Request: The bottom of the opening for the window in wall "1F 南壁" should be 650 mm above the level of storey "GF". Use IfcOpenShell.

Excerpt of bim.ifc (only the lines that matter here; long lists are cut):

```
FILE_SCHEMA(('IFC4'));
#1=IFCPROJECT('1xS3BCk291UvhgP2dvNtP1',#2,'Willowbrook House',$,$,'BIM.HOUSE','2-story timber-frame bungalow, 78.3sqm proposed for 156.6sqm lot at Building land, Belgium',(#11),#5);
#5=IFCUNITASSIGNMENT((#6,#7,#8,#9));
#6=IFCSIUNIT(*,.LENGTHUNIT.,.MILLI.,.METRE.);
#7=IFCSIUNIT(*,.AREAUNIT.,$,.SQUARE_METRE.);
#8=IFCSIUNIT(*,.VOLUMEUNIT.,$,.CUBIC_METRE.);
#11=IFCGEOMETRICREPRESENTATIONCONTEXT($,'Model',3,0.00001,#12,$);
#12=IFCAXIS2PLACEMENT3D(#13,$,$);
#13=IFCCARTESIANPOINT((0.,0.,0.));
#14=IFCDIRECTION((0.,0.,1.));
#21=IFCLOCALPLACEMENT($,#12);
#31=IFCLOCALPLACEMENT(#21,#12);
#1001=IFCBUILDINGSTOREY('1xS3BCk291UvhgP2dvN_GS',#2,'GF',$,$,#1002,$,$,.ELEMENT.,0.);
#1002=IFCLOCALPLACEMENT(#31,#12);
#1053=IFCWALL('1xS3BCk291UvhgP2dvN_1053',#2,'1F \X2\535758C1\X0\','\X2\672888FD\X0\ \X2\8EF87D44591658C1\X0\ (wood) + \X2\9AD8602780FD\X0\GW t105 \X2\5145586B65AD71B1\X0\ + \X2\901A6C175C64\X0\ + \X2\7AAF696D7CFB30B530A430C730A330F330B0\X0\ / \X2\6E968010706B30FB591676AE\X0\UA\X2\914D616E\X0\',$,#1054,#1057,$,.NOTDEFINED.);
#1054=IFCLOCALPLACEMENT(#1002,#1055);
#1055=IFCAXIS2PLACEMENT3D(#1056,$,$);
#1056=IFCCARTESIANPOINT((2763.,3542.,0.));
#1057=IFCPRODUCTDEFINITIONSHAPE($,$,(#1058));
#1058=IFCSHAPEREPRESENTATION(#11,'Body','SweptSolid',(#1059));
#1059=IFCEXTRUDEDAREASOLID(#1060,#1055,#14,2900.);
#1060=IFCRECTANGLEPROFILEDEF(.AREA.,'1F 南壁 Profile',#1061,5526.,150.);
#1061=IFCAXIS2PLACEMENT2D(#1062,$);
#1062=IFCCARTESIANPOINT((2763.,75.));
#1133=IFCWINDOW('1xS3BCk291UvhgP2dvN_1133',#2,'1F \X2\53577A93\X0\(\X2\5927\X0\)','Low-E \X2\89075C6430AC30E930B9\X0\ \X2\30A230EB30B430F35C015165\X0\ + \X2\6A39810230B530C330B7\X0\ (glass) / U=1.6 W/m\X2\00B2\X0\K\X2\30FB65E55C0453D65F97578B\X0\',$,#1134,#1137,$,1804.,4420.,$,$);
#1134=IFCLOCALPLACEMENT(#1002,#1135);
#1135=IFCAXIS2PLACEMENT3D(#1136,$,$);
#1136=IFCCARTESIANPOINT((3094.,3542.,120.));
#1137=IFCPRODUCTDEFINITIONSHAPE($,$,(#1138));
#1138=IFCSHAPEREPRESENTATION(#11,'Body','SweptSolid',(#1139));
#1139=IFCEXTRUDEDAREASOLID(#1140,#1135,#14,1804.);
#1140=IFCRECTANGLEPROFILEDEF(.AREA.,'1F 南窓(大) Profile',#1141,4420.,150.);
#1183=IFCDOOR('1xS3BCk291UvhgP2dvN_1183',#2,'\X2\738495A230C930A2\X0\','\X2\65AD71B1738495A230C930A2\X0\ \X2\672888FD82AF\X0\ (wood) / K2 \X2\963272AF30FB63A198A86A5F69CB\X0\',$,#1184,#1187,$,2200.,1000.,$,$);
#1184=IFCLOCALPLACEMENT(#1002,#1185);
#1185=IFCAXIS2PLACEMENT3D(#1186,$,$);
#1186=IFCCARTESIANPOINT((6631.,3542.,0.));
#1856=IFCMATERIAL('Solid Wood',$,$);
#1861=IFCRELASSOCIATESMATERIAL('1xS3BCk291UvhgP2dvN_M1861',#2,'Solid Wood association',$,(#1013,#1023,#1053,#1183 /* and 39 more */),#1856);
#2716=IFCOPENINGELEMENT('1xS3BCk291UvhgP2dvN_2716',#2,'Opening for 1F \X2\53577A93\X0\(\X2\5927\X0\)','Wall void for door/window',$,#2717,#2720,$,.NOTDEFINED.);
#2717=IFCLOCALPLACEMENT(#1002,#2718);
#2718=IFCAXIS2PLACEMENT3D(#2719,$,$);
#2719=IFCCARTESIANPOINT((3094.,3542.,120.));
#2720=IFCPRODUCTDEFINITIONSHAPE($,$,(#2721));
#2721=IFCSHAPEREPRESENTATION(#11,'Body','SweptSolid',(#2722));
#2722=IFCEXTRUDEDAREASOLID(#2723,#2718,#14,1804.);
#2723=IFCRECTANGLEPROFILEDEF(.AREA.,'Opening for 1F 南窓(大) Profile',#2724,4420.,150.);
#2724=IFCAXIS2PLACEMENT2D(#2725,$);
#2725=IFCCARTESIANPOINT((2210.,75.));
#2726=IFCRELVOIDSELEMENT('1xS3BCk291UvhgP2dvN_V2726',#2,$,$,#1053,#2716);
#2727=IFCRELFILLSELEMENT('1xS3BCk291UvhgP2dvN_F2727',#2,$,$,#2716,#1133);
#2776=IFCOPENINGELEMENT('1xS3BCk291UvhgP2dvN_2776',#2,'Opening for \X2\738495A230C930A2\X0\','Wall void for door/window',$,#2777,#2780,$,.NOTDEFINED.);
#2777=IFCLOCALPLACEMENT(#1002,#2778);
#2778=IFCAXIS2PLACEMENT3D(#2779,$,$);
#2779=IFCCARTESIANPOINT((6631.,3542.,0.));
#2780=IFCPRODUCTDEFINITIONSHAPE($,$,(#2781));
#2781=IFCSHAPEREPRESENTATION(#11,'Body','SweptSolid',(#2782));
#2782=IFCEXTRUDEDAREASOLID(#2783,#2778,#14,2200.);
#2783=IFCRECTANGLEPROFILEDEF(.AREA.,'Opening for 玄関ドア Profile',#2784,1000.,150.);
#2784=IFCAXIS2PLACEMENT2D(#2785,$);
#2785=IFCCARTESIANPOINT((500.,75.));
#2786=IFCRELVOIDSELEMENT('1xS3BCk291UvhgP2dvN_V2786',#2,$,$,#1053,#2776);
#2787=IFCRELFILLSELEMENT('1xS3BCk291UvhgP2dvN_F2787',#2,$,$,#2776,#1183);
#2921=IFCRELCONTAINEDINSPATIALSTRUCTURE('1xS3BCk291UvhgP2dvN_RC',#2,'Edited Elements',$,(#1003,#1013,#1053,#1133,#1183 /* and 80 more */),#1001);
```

```python
import numpy as np
import ifcopenshell
import ifcopenshell.api.geometry
import ifcopenshell.geom
import ifcopenshell.util.element
import ifcopenshell.util.placement
import ifcopenshell.util.shape
import ifcopenshell.util.unit

model = ifcopenshell.open("bim.ifc")
unit_scale = ifcopenshell.util.unit.calculate_unit_scale(model)

window = model.by_guid("1xS3BCk291UvhgP2dvN_1133")
opening = window.FillsVoids[0].RelatingOpeningElement
storey = ifcopenshell.util.element.get_container(window, ifc_class="IfcBuildingStorey")
level = ifcopenshell.util.placement.get_local_placement(storey.ObjectPlacement)[2, 3]

# The opening's origin need not be at the sill, so measure its lowest point.
shape = ifcopenshell.geom.create_shape(ifcopenshell.geom.settings(), opening)
bottom = ifcopenshell.util.shape.get_shape_bottom_elevation(shape, shape.geometry) / unit_scale
dz = level + 0.65 / unit_scale - bottom

shift = np.array([0.0, 0.0, dz])
# The window is not placed relative to its opening, so move both.
for product in (opening, window):
    matrix = ifcopenshell.util.placement.get_local_placement(product.ObjectPlacement)
    matrix[:3, 3] += shift
    ifcopenshell.api.geometry.edit_object_placement(model, product=product, matrix=matrix, is_si=False)

print(f"moved by {dz * unit_scale:+.3f} m")

model.write("bim_rev.ifc")
```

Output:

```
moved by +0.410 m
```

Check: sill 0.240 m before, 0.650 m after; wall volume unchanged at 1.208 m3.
